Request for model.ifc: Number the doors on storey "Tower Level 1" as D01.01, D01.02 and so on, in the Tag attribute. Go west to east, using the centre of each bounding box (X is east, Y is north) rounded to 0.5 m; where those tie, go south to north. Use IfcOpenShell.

First a look at what the model holds.

```python
import ifcopenshell
import ifcopenshell.util.element
import ifcopenshell.util.placement

model = ifcopenshell.open("model.ifc")
print(model.schema)
storey = next(s for s in model.by_type("IfcBuildingStorey") if s.Name == "Tower Level 1")
doors = [e for e in ifcopenshell.util.element.get_decomposition(storey) if e.is_a("IfcDoor")]
for e in sorted(doors, key=lambda e: e.id()):
    origin = ifcopenshell.util.placement.get_local_placement(e.ObjectPlacement)[:3, 3]
    print(e.id(), e.Tag, e.Name, origin.round(2) + 0.0, sep=" | ")
```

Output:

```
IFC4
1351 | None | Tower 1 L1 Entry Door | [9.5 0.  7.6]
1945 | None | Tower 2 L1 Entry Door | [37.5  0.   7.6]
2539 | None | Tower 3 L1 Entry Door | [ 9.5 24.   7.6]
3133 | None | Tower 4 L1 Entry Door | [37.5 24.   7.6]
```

```python
import ifcopenshell
import ifcopenshell.geom
import ifcopenshell.util.element
import ifcopenshell.util.shape

model = ifcopenshell.open("model.ifc")
settings = ifcopenshell.geom.settings()
settings.set("use-world-coords", True)


def centre(element):
    shape = ifcopenshell.geom.create_shape(settings, element)
    return ifcopenshell.util.shape.get_bbox_centroid(shape.geometry)


storey = next(s for s in model.by_type("IfcBuildingStorey") if s.Name == "Tower Level 1")
doors = [e for e in ifcopenshell.util.element.get_decomposition(storey) if e.is_a("IfcDoor")]

# Insertion points can sit at a corner or the storey origin, so sort by the geometry (in metres).
centres = {e: centre(e) for e in doors}
doors.sort(key=lambda e: (round(centres[e][0] / 0.5), centres[e][1]))

for i, e in enumerate(doors, start=1):
    number = f"D01.{i:02d}"
    e.Tag = number
    print(e.id(), number)

model.write("model_updated.ifc")
```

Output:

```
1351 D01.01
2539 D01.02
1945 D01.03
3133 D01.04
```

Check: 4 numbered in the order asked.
